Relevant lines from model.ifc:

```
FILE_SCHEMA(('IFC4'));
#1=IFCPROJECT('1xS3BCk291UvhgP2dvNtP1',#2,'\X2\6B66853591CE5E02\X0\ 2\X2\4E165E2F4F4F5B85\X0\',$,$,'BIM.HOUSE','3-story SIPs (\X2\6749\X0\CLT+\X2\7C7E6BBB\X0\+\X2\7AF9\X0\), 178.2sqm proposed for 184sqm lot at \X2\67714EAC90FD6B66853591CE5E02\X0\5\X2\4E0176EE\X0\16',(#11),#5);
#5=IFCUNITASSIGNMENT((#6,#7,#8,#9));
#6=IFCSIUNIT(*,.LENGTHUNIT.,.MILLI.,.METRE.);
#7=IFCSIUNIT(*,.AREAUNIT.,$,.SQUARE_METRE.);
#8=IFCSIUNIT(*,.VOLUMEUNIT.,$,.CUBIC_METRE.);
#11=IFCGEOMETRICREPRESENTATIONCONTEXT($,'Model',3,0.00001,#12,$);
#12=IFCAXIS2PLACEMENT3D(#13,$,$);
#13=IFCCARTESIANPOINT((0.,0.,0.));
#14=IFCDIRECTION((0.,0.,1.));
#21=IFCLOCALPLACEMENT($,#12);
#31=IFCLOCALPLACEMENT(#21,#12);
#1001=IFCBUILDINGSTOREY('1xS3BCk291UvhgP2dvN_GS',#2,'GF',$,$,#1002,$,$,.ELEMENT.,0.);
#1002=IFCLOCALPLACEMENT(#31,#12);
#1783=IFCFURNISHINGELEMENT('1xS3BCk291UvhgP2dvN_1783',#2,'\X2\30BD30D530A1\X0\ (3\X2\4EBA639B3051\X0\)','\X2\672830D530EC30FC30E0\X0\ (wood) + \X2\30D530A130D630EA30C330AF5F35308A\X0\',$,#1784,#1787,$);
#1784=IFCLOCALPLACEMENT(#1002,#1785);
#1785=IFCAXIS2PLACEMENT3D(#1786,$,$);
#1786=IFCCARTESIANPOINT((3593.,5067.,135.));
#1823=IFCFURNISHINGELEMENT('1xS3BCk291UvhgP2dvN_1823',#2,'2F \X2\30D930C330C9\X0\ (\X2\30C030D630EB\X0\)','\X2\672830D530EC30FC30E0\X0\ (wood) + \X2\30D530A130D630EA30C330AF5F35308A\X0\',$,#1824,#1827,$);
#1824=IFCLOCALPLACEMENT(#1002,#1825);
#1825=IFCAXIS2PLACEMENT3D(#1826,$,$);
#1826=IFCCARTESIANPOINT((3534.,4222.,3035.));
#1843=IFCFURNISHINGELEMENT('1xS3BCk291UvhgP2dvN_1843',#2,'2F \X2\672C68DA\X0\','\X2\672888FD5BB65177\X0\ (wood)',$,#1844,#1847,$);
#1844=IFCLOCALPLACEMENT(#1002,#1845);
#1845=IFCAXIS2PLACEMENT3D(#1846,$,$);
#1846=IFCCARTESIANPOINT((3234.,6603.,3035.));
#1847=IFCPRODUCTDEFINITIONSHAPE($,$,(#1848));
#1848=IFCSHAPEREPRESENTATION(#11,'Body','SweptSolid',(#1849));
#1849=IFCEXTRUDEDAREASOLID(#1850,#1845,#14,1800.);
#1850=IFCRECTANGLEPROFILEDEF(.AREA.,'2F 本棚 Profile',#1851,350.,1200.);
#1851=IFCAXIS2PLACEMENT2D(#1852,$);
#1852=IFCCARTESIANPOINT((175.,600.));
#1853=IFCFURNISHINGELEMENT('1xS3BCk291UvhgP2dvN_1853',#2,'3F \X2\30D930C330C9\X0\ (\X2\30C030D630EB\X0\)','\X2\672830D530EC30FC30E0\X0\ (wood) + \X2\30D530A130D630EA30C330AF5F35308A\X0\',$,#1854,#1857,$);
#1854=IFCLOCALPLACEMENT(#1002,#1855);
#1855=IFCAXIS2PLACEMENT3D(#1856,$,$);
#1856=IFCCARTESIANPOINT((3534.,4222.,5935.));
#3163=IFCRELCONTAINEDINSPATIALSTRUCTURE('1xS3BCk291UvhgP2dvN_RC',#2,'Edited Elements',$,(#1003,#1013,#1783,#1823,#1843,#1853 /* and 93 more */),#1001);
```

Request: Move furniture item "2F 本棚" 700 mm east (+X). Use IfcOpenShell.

```python
import ifcopenshell
import ifcopenshell.api.geometry
import ifcopenshell.util.placement
import ifcopenshell.util.unit

model = ifcopenshell.open("model.ifc")
unit_scale = ifcopenshell.util.unit.calculate_unit_scale(model)

item = model.by_id(1843)
matrix = ifcopenshell.util.placement.get_local_placement(item.ObjectPlacement)
matrix[0, 3] += 0.7 / unit_scale
ifcopenshell.api.geometry.edit_object_placement(model, product=item, matrix=matrix, is_si=False)

print(ifcopenshell.util.placement.get_local_placement(item.ObjectPlacement).round(3) + 0.0)

model.write("model_edited.ifc")
```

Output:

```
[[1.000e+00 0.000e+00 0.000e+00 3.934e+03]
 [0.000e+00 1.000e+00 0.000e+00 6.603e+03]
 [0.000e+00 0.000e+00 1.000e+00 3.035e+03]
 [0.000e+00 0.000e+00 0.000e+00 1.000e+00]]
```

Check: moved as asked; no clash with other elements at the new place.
